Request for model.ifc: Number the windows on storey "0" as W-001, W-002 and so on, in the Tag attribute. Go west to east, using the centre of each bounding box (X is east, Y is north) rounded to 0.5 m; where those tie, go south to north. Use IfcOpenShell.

First a look at what the model holds.

```python
import ifcopenshell
import ifcopenshell.util.element
import ifcopenshell.util.placement

model = ifcopenshell.open("model.ifc")
print(model.schema)
storey = next(s for s in model.by_type("IfcBuildingStorey") if s.Name == "0")
windows = [e for e in ifcopenshell.util.element.get_decomposition(storey) if e.is_a("IfcWindow")]
for e in sorted(windows, key=lambda e: e.id()):
    origin = ifcopenshell.util.placement.get_local_placement(e.ObjectPlacement)[:3, 3]
    print(e.id(), e.Tag, e.Name, origin.round(2) + 0.0, sep=" | ")
```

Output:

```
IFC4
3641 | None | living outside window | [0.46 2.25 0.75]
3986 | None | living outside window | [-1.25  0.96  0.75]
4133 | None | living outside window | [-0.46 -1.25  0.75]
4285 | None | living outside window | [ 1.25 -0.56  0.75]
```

```python
import ifcopenshell
import ifcopenshell.geom
import ifcopenshell.util.element
import ifcopenshell.util.shape

model = ifcopenshell.open("model.ifc")
settings = ifcopenshell.geom.settings()
settings.set("use-world-coords", True)


def centre(element):
    shape = ifcopenshell.geom.create_shape(settings, element)
    return ifcopenshell.util.shape.get_bbox_centroid(shape.geometry)


storey = next(s for s in model.by_type("IfcBuildingStorey") if s.Name == "0")
windows = [e for e in ifcopenshell.util.element.get_decomposition(storey) if e.is_a("IfcWindow")]

# Insertion points can sit at a corner or the storey origin, so sort by the geometry (in metres).
centres = {e: centre(e) for e in windows}
windows.sort(key=lambda e: (round(centres[e][0] / 0.5), centres[e][1]))

for i, e in enumerate(windows, start=1):
    number = f"W-0{i:02d}"
    e.Tag = number
    print(e.id(), number)

model.write("model_rev.ifc")
```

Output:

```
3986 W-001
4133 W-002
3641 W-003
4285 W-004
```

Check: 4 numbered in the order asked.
